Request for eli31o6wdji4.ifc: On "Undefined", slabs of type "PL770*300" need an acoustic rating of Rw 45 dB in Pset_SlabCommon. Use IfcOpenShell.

First a look at what the model holds.

```python
import ifcopenshell
import ifcopenshell.util.element

model = ifcopenshell.open("eli31o6wdji4.ifc")
print(model.schema)
storey = next(s for s in model.by_type("IfcBuildingStorey") if s.Name == "Undefined")
slabs = [e for e in ifcopenshell.util.element.get_decomposition(storey) if e.is_a("IfcSlab")]
seen = {}
for e in slabs:
    element_type = ifcopenshell.util.element.get_type(e)
    key = (element_type.Name if element_type != e and element_type else None, ifcopenshell.util.element.get_pset(e, "Pset_SlabCommon", "AcousticRating"))
    seen[key] = seen.get(key, 0) + 1
for (name, value), count in sorted(seen.items(), key=str):
    print(count, "x", name, "|", value)
```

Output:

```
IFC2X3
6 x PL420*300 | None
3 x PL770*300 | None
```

```python
import ifcopenshell
import ifcopenshell.api.pset
import ifcopenshell.util.element

model = ifcopenshell.open("eli31o6wdji4.ifc")

storey = next(s for s in model.by_type("IfcBuildingStorey") if s.Name == "Undefined")
slabs = [e for e in ifcopenshell.util.element.get_decomposition(storey) if e.is_a("IfcSlab")]

count = 0
for e in slabs:
    element_type = ifcopenshell.util.element.get_type(e)
    if element_type in (None, e) or element_type.Name != "PL770*300":
        continue
    found = ifcopenshell.util.element.get_pset(e, "Pset_SlabCommon", should_inherit=False)
    if found:
        pset = model.by_id(found["id"])
        if len(ifcopenshell.util.element.get_elements_by_pset(pset)) > 1:
            pset = ifcopenshell.api.pset.unshare_pset(model, products=[e], pset=pset)[0]
    else:
        pset = ifcopenshell.api.pset.add_pset(model, product=e, name="Pset_SlabCommon")
    ifcopenshell.api.pset.edit_pset(model, pset=pset, properties={"AcousticRating": "Rw 45 dB"})
    count += 1

print(count, "slabs updated")

model.write("eli31o6wdji4_updated.ifc")
```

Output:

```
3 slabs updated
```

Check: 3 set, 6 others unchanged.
